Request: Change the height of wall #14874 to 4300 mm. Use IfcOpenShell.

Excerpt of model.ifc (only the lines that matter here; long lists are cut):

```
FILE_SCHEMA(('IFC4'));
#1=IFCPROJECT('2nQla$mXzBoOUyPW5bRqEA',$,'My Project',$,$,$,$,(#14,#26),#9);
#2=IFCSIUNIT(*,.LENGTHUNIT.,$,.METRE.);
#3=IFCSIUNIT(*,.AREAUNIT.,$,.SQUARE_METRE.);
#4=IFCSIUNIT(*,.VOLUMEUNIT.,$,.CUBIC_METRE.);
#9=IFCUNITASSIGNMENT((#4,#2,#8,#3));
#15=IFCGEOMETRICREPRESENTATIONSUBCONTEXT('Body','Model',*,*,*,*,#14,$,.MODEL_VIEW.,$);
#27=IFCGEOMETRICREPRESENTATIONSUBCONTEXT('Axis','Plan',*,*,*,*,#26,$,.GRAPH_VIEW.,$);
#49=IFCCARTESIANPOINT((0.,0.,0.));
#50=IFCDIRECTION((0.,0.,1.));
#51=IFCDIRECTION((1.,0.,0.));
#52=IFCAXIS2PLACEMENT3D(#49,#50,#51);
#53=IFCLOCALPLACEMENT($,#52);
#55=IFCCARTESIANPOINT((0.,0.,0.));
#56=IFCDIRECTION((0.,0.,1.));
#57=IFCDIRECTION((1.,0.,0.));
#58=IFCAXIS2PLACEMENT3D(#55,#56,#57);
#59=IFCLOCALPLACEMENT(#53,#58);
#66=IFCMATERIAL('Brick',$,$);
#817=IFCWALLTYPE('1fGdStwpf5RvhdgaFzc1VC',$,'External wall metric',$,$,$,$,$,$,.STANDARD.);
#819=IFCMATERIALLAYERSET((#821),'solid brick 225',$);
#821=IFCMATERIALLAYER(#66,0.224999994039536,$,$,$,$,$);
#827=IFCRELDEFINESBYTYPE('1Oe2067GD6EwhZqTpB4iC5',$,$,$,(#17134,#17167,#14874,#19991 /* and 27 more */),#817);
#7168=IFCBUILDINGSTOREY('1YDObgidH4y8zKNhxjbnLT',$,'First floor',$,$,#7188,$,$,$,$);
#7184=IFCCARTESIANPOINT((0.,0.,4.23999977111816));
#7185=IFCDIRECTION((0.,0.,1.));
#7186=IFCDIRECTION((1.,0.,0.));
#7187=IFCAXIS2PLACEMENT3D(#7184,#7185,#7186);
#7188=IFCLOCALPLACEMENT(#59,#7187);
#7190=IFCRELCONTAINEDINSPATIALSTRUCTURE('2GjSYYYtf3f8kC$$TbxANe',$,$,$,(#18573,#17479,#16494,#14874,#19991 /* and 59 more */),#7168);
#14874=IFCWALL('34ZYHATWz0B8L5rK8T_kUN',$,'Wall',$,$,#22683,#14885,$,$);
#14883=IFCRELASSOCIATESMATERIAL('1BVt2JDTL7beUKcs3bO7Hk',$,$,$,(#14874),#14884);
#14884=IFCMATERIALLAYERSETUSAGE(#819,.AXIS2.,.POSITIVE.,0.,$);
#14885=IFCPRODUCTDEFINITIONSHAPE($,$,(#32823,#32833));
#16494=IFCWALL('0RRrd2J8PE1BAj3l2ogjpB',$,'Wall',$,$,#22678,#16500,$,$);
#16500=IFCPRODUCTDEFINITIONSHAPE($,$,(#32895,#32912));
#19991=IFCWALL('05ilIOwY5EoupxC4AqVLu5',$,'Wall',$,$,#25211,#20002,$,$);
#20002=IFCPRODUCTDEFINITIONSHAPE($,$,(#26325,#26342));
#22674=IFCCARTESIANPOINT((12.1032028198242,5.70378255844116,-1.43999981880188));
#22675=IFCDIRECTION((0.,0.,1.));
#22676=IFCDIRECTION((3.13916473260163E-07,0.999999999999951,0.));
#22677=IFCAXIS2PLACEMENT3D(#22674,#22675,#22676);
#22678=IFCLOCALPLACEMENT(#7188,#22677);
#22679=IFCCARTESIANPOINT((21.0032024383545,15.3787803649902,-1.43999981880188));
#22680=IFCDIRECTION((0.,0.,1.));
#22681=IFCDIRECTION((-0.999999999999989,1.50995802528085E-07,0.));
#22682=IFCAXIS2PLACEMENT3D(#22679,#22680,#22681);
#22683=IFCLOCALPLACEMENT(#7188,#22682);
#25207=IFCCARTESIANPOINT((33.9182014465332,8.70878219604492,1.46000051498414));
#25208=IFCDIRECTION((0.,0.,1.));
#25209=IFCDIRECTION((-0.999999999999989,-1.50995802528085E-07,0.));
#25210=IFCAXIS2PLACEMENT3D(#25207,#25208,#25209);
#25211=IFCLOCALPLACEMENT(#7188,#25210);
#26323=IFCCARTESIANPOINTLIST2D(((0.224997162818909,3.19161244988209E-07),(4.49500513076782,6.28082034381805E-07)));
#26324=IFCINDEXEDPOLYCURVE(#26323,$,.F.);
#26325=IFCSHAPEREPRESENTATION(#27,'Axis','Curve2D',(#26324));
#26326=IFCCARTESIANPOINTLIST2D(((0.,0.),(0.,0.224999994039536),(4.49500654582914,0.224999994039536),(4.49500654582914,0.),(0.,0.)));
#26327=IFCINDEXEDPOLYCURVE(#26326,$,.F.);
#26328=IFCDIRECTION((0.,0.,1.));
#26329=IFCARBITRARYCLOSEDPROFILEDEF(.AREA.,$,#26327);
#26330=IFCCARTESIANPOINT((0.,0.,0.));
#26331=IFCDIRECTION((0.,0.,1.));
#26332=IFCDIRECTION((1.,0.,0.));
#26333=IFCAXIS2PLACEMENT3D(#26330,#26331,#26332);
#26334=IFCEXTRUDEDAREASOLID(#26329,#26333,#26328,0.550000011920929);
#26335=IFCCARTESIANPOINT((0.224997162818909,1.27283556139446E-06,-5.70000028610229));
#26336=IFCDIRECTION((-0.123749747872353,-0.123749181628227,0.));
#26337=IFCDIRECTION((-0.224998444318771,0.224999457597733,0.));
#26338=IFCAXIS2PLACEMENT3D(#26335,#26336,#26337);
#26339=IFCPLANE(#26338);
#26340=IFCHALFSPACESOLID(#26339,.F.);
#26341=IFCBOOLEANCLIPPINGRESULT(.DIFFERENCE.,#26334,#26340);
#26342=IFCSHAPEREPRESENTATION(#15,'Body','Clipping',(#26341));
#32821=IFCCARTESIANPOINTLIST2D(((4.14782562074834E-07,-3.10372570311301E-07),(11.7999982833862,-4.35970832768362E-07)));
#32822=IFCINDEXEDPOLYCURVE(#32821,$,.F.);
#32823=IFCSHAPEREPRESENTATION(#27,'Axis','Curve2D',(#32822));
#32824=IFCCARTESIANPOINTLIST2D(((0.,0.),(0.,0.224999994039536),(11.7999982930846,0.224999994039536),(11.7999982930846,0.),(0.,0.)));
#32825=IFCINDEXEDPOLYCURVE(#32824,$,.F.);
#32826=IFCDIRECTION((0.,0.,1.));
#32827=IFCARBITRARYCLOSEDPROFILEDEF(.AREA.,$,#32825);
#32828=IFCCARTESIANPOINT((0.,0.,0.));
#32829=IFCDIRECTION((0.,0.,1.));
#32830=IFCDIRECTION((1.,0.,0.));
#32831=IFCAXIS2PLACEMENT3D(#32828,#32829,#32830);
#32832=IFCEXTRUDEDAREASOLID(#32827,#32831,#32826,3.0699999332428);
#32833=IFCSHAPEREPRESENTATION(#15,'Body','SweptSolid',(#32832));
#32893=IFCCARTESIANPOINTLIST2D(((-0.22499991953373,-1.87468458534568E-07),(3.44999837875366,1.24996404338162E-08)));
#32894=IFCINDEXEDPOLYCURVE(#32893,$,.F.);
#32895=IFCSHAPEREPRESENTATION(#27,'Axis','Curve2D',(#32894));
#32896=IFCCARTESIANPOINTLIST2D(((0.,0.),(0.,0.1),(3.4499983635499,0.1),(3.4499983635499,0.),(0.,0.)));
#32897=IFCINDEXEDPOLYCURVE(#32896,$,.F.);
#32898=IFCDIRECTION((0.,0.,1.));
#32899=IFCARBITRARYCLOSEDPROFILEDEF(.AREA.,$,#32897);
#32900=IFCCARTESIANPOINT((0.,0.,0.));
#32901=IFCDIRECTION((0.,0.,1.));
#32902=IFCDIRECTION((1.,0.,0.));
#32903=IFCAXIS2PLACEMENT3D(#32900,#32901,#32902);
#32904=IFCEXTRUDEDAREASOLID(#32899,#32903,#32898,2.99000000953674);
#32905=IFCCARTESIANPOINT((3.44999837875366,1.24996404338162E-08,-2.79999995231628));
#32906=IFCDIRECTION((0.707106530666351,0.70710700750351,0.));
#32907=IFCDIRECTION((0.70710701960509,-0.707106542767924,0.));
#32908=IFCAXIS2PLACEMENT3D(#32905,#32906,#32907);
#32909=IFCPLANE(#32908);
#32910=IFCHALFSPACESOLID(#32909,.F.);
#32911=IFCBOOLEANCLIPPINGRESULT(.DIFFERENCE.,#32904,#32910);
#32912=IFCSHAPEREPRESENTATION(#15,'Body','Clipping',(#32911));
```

```python
import ifcopenshell
import ifcopenshell.geom
import ifcopenshell.util.representation
import ifcopenshell.util.shape

model = ifcopenshell.open("model.ifc")
settings = ifcopenshell.geom.settings()


def volume(element):
    """Net volume in cubic metres, openings subtracted."""
    shape = ifcopenshell.geom.create_shape(settings, element)
    return ifcopenshell.util.shape.get_volume(shape.geometry)


wall = model.by_guid("34ZYHATWz0B8L5rK8T_kUN")
before = volume(wall)

body = ifcopenshell.util.representation.get_representation(wall, "Model", "Body")
solid = body.Items[0]
old_height = solid.Depth
solid.Depth = 4.3
after = volume(wall)

print(f"height {old_height:g} -> {solid.Depth:g}, volume {before:.3f} -> {after:.3f} m3")

model.write("model_rev.ifc")
```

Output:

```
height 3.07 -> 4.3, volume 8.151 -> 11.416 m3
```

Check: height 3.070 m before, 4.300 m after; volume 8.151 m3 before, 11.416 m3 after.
